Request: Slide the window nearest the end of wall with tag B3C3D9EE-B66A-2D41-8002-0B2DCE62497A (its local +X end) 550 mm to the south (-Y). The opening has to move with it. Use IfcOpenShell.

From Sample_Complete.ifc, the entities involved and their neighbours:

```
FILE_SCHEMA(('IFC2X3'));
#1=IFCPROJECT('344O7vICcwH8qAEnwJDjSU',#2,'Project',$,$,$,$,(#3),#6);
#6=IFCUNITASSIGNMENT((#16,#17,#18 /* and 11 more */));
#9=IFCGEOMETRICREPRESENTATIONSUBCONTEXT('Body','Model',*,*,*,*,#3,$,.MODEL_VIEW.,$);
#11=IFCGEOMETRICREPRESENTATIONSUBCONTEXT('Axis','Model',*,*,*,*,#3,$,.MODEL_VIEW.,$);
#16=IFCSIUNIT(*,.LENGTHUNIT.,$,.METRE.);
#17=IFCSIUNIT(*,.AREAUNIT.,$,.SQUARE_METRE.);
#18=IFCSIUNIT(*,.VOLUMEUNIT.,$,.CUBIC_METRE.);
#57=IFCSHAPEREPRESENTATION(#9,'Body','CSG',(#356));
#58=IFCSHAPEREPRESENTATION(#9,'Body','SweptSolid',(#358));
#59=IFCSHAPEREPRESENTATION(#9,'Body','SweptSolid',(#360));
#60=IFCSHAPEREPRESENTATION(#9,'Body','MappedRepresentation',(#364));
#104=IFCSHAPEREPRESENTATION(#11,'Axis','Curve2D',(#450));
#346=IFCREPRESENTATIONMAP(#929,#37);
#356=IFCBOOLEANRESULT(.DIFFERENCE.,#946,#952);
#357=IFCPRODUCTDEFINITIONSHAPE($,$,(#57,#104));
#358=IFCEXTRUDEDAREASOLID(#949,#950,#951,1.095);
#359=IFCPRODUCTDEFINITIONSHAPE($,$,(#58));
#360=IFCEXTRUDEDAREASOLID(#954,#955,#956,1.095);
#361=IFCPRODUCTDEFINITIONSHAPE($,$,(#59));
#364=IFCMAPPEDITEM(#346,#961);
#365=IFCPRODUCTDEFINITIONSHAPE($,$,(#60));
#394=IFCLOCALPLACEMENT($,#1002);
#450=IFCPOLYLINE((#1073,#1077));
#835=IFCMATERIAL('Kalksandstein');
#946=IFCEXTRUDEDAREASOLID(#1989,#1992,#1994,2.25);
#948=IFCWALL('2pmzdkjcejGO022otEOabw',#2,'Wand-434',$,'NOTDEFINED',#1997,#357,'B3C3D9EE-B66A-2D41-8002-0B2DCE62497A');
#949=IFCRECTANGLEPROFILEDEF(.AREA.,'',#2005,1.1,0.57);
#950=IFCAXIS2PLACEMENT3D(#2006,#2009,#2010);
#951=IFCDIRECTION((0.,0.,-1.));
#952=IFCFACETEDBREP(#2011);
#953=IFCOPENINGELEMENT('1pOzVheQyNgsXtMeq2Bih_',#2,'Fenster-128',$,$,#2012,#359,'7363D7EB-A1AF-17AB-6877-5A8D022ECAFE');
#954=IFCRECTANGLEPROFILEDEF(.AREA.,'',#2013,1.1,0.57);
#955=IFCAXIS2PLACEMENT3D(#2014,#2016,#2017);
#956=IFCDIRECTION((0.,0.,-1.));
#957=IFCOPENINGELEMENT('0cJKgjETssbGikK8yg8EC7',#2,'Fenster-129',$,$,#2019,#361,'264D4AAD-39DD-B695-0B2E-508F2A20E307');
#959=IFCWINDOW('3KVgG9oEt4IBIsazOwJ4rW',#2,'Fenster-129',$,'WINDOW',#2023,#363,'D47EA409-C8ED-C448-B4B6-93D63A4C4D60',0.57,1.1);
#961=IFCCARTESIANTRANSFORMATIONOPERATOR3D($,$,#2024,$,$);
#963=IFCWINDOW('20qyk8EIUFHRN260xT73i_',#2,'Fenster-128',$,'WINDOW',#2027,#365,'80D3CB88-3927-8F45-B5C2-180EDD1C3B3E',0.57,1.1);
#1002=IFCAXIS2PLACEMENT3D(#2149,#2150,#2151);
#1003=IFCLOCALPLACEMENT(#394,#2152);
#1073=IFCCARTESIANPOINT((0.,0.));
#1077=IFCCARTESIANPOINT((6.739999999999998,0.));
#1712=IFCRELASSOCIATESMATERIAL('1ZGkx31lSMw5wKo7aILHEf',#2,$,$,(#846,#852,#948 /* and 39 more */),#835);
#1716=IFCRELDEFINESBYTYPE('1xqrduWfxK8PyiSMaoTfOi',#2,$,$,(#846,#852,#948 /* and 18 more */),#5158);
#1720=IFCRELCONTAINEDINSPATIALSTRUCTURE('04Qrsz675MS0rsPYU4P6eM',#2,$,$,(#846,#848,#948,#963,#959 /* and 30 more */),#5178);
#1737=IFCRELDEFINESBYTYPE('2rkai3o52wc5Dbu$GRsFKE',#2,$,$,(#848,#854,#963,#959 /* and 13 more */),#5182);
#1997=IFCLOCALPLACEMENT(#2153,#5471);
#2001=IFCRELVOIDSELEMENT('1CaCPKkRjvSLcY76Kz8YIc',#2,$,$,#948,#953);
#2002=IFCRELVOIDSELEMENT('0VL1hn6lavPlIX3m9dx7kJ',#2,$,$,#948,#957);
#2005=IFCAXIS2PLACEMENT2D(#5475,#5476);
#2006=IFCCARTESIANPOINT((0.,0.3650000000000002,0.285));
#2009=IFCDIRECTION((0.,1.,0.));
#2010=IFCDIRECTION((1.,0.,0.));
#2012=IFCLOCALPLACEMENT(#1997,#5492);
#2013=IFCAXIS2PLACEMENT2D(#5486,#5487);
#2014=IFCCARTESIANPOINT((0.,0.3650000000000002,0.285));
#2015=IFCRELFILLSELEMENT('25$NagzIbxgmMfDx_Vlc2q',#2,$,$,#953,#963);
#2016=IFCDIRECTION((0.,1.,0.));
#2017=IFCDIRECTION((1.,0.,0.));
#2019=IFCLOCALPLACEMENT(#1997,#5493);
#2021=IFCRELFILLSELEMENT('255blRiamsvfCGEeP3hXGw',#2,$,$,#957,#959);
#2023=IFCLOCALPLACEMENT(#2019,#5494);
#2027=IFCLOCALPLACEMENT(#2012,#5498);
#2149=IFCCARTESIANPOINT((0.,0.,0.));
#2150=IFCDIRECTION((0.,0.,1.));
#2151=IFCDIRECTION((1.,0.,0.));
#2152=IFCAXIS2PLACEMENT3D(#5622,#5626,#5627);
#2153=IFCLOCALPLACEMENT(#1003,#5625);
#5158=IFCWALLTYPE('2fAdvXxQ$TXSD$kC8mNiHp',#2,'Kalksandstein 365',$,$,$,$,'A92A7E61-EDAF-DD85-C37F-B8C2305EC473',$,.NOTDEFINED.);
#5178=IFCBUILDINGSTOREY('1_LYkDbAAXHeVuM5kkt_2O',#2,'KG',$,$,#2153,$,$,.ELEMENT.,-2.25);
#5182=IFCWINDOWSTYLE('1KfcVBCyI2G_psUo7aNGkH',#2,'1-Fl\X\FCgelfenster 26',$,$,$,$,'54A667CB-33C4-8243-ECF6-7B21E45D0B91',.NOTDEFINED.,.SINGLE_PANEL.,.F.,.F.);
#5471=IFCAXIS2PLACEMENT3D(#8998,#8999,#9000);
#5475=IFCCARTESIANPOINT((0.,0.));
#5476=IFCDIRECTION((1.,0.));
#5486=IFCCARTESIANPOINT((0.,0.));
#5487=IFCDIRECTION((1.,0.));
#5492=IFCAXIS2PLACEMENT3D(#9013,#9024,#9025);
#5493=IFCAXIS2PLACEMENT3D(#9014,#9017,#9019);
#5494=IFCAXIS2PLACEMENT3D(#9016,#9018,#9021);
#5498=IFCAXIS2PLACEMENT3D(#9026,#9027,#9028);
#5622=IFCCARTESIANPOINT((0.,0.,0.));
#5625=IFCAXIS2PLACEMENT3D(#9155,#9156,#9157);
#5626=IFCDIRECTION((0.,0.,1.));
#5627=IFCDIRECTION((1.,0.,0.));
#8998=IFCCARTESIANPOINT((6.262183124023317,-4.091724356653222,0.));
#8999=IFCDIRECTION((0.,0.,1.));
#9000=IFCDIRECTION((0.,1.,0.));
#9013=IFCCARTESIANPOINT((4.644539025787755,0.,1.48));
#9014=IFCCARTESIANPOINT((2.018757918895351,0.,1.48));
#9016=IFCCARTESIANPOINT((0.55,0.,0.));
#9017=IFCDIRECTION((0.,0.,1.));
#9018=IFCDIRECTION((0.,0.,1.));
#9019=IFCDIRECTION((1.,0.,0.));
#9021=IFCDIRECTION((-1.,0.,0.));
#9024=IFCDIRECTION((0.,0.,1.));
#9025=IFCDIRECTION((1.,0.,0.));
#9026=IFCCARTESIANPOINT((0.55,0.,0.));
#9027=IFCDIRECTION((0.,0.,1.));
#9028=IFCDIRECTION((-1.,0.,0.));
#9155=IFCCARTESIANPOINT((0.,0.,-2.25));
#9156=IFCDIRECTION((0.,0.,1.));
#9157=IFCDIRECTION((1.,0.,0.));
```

```python
import ifcopenshell
import ifcopenshell.api.geometry
import ifcopenshell.util.placement
import ifcopenshell.util.unit

model = ifcopenshell.open("Sample_Complete.ifc")
unit_scale = ifcopenshell.util.unit.calculate_unit_scale(model)

window = model.by_guid("20qyk8EIUFHRN260xT73i_")
opening = window.FillsVoids[0].RelatingOpeningElement
wall = opening.VoidsElements[0].RelatingBuildingElement

wall_matrix = ifcopenshell.util.placement.get_local_placement(wall.ObjectPlacement)
shift = wall_matrix[:3, 0] * -0.55 / unit_scale
before = ifcopenshell.util.placement.get_local_placement(window.ObjectPlacement)[:3, 3].copy()

# The window is placed relative to its opening, so it follows when the opening moves.
matrix = ifcopenshell.util.placement.get_local_placement(opening.ObjectPlacement)
matrix[:3, 3] += shift
ifcopenshell.api.geometry.edit_object_placement(
    model, product=opening, matrix=matrix, is_si=False, should_transform_children=True
)

after = ifcopenshell.util.placement.get_local_placement(window.ObjectPlacement)[:3, 3]
print("window moved by", (after - before).round(3) + 0.0)

model.write("Sample_Complete_rev.ifc")
```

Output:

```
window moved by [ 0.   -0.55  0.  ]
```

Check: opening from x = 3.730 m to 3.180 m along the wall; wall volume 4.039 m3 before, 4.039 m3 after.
